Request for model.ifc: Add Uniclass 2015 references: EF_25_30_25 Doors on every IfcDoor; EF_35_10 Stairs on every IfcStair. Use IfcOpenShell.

First a look at what the model holds.

```python
import ifcopenshell

model = ifcopenshell.open("model.ifc")
print(model.schema)
print("classifications:", [c.Name for c in model.by_type("IfcClassification")])
for ifc_class in ("IfcDoor", "IfcRoof", "IfcStair", "IfcWall", "IfcWindow"):
    print(ifc_class, len(model.by_type(ifc_class)))
```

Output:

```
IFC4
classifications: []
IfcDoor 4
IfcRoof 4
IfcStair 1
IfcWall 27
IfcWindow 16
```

```python
import ifcopenshell
import ifcopenshell.api.classification

model = ifcopenshell.open("model.ifc")

system = ifcopenshell.api.classification.add_classification(model, classification="Uniclass 2015")

codes = {
    "IfcDoor": ("EF_25_30_25", "Doors"),
    "IfcStair": ("EF_35_10", "Stairs"),
}
for ifc_class, (code, name) in codes.items():
    products = model.by_type(ifc_class)
    ifcopenshell.api.classification.add_reference(
        model, products=products, classification=system, identification=code, name=name
    )
    print(code, len(products))

model.write("model_updated.ifc")
```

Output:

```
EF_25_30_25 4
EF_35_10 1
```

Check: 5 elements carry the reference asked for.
